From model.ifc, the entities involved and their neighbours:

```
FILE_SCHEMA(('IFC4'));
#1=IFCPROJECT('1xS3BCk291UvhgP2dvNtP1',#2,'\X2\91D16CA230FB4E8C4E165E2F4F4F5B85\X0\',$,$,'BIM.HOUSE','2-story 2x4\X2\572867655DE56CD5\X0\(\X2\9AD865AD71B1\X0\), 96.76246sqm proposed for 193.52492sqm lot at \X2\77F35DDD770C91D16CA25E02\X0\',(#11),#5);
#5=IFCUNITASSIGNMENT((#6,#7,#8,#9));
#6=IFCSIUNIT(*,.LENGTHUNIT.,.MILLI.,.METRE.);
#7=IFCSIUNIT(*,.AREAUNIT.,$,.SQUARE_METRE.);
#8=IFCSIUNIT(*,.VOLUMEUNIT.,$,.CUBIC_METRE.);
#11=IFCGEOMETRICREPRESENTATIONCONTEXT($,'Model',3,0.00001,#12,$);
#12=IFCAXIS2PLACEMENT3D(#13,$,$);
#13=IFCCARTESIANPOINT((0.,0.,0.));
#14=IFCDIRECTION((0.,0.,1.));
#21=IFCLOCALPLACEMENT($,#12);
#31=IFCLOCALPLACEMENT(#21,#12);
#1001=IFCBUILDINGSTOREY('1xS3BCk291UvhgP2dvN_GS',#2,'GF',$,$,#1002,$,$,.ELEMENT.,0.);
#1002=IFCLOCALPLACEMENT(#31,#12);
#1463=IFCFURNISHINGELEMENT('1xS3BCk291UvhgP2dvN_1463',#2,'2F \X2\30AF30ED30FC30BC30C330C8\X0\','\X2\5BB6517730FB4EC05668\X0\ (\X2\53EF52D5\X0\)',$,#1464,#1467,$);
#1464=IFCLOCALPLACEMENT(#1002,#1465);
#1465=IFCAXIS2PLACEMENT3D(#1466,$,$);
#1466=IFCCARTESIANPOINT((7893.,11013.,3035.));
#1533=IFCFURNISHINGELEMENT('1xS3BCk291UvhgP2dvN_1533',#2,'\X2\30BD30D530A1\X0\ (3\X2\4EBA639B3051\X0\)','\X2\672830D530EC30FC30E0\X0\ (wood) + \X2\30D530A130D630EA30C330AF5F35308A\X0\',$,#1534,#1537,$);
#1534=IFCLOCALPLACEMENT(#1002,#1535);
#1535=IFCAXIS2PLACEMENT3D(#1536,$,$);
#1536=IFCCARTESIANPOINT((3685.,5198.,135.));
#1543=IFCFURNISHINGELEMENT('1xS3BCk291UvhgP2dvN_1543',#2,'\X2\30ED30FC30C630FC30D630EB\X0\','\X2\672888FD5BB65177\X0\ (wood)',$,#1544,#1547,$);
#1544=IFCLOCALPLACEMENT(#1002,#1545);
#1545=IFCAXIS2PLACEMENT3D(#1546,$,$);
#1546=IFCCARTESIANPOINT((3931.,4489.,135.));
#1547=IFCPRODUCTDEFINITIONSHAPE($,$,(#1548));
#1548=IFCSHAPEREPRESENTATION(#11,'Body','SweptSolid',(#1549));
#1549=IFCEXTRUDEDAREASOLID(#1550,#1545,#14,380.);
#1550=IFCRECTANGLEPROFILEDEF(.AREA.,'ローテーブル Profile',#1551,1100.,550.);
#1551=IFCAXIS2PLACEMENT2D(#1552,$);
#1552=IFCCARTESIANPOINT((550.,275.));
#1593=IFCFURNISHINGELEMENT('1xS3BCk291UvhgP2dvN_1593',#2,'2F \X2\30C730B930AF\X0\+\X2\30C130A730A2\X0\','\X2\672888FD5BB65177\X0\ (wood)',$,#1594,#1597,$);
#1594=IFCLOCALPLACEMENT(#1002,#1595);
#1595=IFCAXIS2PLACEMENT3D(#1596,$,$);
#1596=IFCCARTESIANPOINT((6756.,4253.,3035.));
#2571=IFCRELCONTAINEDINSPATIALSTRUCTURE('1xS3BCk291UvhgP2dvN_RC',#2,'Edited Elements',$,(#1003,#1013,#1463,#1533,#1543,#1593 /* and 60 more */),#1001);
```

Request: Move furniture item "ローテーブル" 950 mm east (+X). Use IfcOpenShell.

```python
import ifcopenshell
import ifcopenshell.api.geometry
import ifcopenshell.util.placement

model = ifcopenshell.open("model.ifc")

item = model.by_guid("1xS3BCk291UvhgP2dvN_1543")
matrix = ifcopenshell.util.placement.get_local_placement(item.ObjectPlacement)
matrix[0, 3] += 950.0
ifcopenshell.api.geometry.edit_object_placement(model, product=item, matrix=matrix, is_si=False)

print(ifcopenshell.util.placement.get_local_placement(item.ObjectPlacement).round(3) + 0.0)

model.write("model_rev.ifc")
```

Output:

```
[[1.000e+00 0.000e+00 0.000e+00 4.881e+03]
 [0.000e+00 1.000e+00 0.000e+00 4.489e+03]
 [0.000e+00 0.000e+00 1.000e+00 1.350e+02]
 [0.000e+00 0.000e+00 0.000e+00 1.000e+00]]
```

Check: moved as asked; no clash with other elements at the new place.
